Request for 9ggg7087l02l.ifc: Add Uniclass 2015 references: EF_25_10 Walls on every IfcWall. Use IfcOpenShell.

First a look at what the model holds.

```python
import ifcopenshell

model = ifcopenshell.open("9ggg7087l02l.ifc")
print(model.schema)
print("classifications:", [c.Name for c in model.by_type("IfcClassification")])
for ifc_class in ("IfcDoor", "IfcRoof", "IfcStair", "IfcWall", "IfcWindow"):
    print(ifc_class, len(model.by_type(ifc_class)))
```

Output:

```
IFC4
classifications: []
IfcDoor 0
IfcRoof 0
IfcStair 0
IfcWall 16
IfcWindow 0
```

```python
import ifcopenshell
import ifcopenshell.api.classification

model = ifcopenshell.open("9ggg7087l02l.ifc")

system = ifcopenshell.api.classification.add_classification(model, classification="Uniclass 2015")

codes = {
    "IfcWall": ("EF_25_10", "Walls"),
}
for ifc_class, (code, name) in codes.items():
    products = model.by_type(ifc_class)
    ifcopenshell.api.classification.add_reference(
        model, products=products, classification=system, identification=code, name=name
    )
    print(code, len(products))

model.write("9ggg7087l02l_rev.ifc")
```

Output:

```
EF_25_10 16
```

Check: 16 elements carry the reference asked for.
